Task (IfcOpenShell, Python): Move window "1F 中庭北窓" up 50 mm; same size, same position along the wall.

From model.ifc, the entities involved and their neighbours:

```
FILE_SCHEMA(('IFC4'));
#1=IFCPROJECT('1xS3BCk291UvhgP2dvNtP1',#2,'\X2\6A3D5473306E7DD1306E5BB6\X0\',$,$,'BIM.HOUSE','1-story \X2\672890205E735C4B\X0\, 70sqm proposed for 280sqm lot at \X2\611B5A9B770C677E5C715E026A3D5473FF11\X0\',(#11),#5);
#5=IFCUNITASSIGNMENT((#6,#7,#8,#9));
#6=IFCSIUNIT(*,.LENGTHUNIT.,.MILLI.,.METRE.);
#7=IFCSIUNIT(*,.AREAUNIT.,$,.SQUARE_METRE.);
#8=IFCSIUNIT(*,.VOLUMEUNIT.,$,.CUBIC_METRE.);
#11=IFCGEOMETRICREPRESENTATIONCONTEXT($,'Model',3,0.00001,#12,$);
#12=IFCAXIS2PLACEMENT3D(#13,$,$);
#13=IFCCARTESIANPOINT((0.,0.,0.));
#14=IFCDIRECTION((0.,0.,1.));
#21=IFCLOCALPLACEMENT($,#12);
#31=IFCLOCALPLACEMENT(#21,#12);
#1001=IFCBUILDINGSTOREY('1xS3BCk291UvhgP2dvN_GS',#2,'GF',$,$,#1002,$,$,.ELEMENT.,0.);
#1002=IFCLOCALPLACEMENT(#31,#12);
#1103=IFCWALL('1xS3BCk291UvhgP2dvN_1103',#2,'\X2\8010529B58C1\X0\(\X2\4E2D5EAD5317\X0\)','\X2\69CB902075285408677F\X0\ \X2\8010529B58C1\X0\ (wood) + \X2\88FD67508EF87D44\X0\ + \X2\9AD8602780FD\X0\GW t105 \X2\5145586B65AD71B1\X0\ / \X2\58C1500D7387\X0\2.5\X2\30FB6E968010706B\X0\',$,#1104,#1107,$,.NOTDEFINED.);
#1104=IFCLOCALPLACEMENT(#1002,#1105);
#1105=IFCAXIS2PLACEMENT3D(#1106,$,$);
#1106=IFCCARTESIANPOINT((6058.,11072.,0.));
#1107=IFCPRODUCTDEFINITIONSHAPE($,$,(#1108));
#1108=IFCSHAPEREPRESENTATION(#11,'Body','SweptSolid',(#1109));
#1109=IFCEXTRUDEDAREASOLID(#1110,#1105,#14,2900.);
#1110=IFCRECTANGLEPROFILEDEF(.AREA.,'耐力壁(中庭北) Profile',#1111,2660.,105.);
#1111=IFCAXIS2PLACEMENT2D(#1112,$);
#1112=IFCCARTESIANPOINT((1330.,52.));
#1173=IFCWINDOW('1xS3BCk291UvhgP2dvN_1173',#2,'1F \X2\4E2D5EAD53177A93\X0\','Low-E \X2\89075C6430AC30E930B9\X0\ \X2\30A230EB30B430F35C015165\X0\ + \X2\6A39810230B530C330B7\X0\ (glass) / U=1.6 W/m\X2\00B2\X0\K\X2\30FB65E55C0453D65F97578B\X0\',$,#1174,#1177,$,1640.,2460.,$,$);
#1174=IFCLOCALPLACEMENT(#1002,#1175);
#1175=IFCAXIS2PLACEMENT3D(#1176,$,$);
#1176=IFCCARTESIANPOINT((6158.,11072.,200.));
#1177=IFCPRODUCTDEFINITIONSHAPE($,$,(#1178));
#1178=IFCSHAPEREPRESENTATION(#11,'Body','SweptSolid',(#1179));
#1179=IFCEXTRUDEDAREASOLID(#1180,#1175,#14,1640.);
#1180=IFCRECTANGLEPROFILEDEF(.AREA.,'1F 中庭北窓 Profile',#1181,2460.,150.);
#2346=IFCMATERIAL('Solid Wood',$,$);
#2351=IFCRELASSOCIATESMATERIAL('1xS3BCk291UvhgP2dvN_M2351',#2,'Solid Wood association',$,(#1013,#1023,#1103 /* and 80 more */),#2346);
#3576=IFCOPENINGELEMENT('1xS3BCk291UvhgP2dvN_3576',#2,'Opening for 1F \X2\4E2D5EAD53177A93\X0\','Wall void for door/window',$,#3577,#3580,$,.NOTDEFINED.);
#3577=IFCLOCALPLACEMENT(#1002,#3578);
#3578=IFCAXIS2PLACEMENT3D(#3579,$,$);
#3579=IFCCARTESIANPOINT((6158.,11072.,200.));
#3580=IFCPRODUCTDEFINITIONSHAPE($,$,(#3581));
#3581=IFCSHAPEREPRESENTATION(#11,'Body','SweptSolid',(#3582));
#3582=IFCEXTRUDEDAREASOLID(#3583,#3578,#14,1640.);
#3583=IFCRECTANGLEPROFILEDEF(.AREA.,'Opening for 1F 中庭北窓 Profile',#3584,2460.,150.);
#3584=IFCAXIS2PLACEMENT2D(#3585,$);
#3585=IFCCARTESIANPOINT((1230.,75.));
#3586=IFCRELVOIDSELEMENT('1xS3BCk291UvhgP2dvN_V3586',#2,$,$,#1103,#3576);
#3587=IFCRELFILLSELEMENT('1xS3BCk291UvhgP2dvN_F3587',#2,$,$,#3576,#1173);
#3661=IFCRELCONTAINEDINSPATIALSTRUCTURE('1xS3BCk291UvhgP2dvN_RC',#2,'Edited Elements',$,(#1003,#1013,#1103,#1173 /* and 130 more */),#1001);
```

```python
import numpy as np
import ifcopenshell
import ifcopenshell.api.geometry
import ifcopenshell.util.placement
import ifcopenshell.util.unit

model = ifcopenshell.open("model.ifc")
unit_scale = ifcopenshell.util.unit.calculate_unit_scale(model)

window = model.by_guid("1xS3BCk291UvhgP2dvN_1173")
opening = window.FillsVoids[0].RelatingOpeningElement
dz = 0.05 / unit_scale

shift = np.array([0.0, 0.0, dz])
# The window is not placed relative to its opening, so move both.
for product in (opening, window):
    matrix = ifcopenshell.util.placement.get_local_placement(product.ObjectPlacement)
    matrix[:3, 3] += shift
    ifcopenshell.api.geometry.edit_object_placement(model, product=product, matrix=matrix, is_si=False)

print(f"moved by {dz * unit_scale:+.3f} m")

model.write("model_edited.ifc")
```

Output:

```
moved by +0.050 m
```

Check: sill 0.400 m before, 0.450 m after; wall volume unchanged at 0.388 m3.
